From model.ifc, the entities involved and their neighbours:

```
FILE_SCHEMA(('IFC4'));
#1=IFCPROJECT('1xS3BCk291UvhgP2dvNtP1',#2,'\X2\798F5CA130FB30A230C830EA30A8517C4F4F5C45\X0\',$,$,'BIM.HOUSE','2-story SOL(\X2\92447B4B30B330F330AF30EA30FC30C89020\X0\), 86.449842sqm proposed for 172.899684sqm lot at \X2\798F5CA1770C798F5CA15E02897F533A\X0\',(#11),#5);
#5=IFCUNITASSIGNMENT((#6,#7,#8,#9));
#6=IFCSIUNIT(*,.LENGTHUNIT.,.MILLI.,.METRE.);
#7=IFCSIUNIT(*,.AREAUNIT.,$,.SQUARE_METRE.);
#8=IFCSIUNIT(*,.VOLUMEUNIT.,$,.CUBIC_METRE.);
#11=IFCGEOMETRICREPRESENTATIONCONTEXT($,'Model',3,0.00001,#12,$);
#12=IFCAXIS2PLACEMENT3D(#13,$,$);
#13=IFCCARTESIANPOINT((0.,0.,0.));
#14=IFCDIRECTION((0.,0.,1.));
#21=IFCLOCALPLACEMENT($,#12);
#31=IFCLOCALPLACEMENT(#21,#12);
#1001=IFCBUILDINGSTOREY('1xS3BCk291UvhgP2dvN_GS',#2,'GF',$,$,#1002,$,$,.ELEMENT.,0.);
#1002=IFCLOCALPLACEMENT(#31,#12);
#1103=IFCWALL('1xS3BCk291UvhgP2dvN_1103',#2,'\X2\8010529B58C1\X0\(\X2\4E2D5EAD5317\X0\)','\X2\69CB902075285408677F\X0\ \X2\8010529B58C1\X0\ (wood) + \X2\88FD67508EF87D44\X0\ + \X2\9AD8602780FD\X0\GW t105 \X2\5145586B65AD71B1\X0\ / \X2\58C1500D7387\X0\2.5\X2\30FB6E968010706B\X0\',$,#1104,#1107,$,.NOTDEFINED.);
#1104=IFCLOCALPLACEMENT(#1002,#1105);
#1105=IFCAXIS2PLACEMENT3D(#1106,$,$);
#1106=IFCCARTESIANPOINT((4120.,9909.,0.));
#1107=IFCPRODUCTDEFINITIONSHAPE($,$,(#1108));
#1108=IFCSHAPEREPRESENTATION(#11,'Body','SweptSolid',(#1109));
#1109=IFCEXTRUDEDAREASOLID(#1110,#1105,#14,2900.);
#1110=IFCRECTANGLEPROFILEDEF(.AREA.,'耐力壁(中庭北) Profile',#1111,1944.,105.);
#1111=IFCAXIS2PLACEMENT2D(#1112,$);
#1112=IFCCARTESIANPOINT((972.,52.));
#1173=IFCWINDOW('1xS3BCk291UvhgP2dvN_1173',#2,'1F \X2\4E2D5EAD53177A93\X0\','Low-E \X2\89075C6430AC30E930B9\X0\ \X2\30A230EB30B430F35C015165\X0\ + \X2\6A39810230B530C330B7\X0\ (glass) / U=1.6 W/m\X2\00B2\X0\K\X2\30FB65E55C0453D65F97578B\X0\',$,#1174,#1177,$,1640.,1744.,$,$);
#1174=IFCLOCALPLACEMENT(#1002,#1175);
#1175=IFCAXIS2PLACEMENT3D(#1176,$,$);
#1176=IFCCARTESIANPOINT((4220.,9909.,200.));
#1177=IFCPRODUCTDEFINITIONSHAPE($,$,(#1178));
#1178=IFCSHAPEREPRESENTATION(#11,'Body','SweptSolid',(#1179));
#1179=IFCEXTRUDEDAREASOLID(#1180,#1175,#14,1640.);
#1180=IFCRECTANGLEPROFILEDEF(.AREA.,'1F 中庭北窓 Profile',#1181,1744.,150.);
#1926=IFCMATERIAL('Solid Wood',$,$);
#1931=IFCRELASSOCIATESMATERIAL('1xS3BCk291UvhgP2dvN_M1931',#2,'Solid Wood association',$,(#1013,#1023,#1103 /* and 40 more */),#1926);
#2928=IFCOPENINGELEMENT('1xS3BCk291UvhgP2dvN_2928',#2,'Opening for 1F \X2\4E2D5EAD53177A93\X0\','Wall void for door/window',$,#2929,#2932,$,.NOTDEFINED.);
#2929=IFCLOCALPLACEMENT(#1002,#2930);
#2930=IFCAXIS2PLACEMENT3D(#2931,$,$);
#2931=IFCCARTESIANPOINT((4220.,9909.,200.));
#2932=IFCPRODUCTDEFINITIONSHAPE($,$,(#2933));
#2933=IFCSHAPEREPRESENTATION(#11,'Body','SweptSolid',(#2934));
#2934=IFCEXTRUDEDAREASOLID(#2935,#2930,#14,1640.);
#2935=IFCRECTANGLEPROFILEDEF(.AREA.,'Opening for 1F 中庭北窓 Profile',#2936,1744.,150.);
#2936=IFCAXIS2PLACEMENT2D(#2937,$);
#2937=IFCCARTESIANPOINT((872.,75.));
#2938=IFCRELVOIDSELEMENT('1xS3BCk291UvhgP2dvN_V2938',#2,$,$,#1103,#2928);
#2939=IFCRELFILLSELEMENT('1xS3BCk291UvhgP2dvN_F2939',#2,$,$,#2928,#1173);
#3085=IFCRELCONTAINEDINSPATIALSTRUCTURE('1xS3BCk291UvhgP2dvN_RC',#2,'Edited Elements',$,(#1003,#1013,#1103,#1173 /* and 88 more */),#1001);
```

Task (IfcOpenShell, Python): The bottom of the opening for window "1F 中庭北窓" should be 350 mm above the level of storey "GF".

```python
import numpy as np
import ifcopenshell
import ifcopenshell.api.geometry
import ifcopenshell.geom
import ifcopenshell.util.element
import ifcopenshell.util.placement
import ifcopenshell.util.shape
import ifcopenshell.util.unit

model = ifcopenshell.open("model.ifc")
unit_scale = ifcopenshell.util.unit.calculate_unit_scale(model)

window = model.by_guid("1xS3BCk291UvhgP2dvN_1173")
opening = window.FillsVoids[0].RelatingOpeningElement
storey = ifcopenshell.util.element.get_container(window, ifc_class="IfcBuildingStorey")
level = ifcopenshell.util.placement.get_local_placement(storey.ObjectPlacement)[2, 3]

# The opening's origin need not be at the sill, so measure its lowest point.
shape = ifcopenshell.geom.create_shape(ifcopenshell.geom.settings(), opening)
bottom = ifcopenshell.util.shape.get_shape_bottom_elevation(shape, shape.geometry) / unit_scale
dz = level + 0.35 / unit_scale - bottom

shift = np.array([0.0, 0.0, dz])
# The window is not placed relative to its opening, so move both.
for product in (opening, window):
    matrix = ifcopenshell.util.placement.get_local_placement(product.ObjectPlacement)
    matrix[:3, 3] += shift
    ifcopenshell.api.geometry.edit_object_placement(model, product=product, matrix=matrix, is_si=False)

print(f"moved by {dz * unit_scale:+.3f} m")

model.write("model_rev.ifc")
```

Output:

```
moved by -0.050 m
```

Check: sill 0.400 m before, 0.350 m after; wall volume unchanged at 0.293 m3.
